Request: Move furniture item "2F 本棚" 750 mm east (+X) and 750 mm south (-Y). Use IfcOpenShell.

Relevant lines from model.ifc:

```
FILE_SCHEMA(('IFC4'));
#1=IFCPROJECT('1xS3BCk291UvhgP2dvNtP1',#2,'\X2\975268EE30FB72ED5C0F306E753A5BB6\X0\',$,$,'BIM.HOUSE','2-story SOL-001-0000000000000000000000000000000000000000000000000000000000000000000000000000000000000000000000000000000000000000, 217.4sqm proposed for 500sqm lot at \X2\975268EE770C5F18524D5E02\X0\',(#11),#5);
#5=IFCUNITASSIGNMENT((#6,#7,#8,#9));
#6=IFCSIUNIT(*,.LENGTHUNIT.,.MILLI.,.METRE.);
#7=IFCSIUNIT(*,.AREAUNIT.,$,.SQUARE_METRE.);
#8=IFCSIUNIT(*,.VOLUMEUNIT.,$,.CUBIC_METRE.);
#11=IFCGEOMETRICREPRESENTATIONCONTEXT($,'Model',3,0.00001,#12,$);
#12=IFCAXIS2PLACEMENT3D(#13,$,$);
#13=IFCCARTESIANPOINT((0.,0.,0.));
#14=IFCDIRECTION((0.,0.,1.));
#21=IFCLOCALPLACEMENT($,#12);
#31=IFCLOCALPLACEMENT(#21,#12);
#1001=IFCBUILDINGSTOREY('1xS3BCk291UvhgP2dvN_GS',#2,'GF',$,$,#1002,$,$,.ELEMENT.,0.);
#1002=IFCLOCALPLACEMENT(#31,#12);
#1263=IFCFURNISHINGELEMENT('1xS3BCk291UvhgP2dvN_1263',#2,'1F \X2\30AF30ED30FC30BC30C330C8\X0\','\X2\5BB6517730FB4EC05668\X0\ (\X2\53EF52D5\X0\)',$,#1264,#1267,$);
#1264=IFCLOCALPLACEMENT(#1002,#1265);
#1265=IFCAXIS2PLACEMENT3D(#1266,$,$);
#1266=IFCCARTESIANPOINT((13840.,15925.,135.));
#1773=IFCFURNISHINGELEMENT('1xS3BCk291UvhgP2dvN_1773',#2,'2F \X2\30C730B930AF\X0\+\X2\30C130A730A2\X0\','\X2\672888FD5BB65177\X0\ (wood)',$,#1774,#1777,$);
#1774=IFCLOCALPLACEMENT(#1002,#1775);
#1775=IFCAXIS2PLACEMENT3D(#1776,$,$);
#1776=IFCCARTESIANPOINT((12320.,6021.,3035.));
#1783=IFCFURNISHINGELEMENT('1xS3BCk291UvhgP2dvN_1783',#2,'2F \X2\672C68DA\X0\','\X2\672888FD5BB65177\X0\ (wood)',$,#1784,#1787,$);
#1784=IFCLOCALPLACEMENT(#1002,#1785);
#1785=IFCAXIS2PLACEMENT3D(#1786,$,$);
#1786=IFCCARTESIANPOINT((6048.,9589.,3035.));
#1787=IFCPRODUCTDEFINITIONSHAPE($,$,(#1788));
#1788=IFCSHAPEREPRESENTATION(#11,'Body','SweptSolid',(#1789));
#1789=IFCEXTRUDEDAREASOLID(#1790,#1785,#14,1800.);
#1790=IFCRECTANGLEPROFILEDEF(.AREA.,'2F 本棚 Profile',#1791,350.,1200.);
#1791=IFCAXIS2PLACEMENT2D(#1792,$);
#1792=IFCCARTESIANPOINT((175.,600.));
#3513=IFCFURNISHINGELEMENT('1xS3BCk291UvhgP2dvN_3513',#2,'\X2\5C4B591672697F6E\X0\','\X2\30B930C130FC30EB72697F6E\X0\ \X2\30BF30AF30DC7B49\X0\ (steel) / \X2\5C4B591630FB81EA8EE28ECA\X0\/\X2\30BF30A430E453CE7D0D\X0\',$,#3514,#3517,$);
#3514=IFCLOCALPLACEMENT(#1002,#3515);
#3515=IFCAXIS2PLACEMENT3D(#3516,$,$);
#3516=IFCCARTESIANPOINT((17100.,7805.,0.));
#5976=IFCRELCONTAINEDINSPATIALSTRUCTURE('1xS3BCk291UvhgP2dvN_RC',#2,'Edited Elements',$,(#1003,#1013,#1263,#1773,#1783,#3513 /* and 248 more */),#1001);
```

```python
import ifcopenshell
import ifcopenshell.api.geometry
import ifcopenshell.util.placement

model = ifcopenshell.open("model.ifc")

item = model.by_guid("1xS3BCk291UvhgP2dvN_1783")
matrix = ifcopenshell.util.placement.get_local_placement(item.ObjectPlacement)
matrix[0, 3] += 750.0
matrix[1, 3] -= 750.0
ifcopenshell.api.geometry.edit_object_placement(model, product=item, matrix=matrix, is_si=False)

print(ifcopenshell.util.placement.get_local_placement(item.ObjectPlacement).round(3) + 0.0)

model.write("model_updated.ifc")
```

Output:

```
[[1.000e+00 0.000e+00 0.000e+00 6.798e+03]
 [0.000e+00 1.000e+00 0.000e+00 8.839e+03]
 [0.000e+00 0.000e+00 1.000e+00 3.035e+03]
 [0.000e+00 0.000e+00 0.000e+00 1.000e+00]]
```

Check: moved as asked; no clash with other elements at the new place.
